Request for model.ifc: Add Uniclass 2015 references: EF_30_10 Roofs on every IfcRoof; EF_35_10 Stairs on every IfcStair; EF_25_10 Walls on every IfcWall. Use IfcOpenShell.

First a look at what the model holds.

```python
import ifcopenshell

model = ifcopenshell.open("model.ifc")
print(model.schema)
print("classifications:", [c.Name for c in model.by_type("IfcClassification")])
for ifc_class in ("IfcDoor", "IfcRoof", "IfcStair", "IfcWall", "IfcWindow"):
    print(ifc_class, len(model.by_type(ifc_class)))
```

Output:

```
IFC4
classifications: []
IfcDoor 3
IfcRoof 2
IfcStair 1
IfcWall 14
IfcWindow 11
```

```python
import ifcopenshell
import ifcopenshell.api.classification

model = ifcopenshell.open("model.ifc")

system = ifcopenshell.api.classification.add_classification(model, classification="Uniclass 2015")

codes = {
    "IfcRoof": ("EF_30_10", "Roofs"),
    "IfcStair": ("EF_35_10", "Stairs"),
    "IfcWall": ("EF_25_10", "Walls"),
}
for ifc_class, (code, name) in codes.items():
    products = model.by_type(ifc_class)
    ifcopenshell.api.classification.add_reference(
        model, products=products, classification=system, identification=code, name=name
    )
    print(code, len(products))

model.write("model-out.ifc")
```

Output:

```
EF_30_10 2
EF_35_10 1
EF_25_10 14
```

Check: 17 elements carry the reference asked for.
